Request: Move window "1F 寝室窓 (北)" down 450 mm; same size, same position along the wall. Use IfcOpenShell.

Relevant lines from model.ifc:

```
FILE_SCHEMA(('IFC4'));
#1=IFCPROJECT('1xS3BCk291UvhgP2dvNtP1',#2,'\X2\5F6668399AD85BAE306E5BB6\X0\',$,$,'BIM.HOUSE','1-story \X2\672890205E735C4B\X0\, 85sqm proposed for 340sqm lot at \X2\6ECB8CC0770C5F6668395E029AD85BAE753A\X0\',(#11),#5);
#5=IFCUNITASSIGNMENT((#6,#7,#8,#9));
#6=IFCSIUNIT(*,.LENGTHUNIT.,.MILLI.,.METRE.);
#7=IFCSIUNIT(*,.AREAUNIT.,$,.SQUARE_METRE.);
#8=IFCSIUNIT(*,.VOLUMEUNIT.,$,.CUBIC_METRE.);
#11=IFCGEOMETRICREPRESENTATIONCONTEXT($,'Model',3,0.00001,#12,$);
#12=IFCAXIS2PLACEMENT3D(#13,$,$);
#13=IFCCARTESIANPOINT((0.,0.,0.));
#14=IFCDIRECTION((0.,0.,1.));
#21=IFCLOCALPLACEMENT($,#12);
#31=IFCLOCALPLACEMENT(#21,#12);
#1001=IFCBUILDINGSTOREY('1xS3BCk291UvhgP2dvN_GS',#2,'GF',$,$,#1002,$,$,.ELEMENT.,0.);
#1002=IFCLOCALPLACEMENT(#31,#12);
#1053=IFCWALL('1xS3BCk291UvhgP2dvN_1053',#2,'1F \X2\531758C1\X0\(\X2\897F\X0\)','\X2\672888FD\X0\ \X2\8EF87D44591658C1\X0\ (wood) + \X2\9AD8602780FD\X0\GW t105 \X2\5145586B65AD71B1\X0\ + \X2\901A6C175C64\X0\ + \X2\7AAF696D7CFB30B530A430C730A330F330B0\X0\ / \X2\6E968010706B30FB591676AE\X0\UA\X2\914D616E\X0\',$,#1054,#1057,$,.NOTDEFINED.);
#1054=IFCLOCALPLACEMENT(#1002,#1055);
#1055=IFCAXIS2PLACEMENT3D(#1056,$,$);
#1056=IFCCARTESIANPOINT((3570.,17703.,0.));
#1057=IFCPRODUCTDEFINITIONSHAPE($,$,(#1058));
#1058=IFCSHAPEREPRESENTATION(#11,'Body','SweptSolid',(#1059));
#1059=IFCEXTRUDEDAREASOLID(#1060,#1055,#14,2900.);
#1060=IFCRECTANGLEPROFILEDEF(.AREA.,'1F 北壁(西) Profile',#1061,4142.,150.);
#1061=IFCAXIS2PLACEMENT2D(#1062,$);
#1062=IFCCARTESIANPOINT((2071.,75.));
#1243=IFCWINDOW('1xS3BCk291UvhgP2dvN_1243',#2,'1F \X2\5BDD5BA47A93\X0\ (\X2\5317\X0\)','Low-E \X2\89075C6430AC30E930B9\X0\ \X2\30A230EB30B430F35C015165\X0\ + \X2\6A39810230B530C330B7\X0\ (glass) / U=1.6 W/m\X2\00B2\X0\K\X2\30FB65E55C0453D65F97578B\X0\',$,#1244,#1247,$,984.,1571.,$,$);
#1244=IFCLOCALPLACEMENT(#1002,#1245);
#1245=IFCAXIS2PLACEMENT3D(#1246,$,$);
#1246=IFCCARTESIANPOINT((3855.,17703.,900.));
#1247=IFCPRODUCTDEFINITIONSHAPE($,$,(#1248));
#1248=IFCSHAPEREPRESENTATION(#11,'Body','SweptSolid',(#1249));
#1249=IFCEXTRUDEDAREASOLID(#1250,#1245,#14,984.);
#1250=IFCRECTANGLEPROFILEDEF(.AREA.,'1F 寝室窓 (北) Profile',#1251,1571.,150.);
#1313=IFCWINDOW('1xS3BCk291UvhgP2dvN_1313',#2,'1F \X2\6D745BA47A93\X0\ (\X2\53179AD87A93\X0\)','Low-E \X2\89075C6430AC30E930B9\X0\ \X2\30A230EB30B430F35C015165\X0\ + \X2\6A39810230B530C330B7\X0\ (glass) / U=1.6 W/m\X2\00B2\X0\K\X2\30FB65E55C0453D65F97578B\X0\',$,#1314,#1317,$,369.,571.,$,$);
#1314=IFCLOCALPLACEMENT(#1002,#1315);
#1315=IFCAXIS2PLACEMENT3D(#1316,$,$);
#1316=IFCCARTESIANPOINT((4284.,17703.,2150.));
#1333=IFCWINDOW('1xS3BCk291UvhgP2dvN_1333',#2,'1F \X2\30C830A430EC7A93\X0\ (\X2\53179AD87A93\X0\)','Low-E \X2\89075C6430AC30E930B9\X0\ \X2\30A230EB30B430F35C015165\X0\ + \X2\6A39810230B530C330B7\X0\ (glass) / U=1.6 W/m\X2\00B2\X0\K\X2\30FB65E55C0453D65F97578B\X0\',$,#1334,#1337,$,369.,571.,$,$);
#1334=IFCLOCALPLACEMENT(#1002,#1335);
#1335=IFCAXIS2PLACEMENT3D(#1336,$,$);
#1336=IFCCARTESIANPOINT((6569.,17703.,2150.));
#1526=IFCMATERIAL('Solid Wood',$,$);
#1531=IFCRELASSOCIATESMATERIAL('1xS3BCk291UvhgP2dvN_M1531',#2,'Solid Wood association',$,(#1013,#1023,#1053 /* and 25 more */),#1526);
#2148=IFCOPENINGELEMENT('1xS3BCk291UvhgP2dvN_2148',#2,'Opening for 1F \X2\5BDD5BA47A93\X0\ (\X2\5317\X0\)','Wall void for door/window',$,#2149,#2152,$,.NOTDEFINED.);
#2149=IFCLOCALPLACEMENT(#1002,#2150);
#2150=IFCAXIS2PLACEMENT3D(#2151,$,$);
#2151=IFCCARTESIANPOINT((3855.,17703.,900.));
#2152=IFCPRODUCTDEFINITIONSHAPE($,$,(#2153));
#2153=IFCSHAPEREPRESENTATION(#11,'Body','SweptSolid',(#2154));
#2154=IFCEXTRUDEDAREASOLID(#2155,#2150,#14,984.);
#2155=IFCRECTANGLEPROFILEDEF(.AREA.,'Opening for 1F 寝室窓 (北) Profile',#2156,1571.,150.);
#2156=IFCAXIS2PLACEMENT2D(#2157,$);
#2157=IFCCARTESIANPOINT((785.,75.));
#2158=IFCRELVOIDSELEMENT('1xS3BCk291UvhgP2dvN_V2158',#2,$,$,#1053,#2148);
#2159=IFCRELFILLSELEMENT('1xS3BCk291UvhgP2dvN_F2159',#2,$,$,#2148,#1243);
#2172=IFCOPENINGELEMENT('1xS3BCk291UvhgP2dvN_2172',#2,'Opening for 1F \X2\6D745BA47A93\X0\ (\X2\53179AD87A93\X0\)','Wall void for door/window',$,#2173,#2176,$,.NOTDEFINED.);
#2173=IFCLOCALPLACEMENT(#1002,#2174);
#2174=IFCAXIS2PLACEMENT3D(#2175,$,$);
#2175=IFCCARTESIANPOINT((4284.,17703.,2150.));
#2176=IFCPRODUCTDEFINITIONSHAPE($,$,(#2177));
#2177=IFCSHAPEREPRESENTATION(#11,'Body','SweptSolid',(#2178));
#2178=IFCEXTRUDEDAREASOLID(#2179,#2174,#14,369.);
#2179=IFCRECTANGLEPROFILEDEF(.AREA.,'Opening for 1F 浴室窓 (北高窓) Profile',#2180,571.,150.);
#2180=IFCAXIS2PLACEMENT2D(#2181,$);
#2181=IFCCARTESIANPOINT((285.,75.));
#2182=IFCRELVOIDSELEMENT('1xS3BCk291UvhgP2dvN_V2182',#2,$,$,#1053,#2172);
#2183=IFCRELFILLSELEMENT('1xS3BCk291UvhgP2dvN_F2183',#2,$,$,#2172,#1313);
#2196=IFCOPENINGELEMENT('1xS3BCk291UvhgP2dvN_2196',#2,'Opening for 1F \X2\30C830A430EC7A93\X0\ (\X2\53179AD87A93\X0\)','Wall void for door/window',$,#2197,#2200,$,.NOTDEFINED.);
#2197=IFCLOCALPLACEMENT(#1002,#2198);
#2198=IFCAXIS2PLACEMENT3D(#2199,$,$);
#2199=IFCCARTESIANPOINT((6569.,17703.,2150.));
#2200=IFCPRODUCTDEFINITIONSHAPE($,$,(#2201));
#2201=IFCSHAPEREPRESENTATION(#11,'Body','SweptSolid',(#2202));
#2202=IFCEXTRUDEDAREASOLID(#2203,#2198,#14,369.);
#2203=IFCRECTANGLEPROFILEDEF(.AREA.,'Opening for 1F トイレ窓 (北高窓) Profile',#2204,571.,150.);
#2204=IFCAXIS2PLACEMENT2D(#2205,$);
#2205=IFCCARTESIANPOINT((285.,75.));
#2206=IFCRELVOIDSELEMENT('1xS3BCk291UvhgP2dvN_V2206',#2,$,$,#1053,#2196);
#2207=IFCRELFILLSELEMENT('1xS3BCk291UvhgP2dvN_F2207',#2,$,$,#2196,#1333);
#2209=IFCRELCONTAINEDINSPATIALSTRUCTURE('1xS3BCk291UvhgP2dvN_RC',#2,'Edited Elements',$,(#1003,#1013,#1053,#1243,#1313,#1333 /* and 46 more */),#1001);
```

```python
import numpy as np
import ifcopenshell
import ifcopenshell.api.geometry
import ifcopenshell.util.placement
import ifcopenshell.util.unit

model = ifcopenshell.open("model.ifc")
unit_scale = ifcopenshell.util.unit.calculate_unit_scale(model)

window = model.by_guid("1xS3BCk291UvhgP2dvN_1243")
opening = window.FillsVoids[0].RelatingOpeningElement
dz = -0.45 / unit_scale

shift = np.array([0.0, 0.0, dz])
# The window is not placed relative to its opening, so move both.
for product in (opening, window):
    matrix = ifcopenshell.util.placement.get_local_placement(product.ObjectPlacement)
    matrix[:3, 3] += shift
    ifcopenshell.api.geometry.edit_object_placement(model, product=product, matrix=matrix, is_si=False)

print(f"moved by {dz * unit_scale:+.3f} m")

model.write("model_v2.ifc")
```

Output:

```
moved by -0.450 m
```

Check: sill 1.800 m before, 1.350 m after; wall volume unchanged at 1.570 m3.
